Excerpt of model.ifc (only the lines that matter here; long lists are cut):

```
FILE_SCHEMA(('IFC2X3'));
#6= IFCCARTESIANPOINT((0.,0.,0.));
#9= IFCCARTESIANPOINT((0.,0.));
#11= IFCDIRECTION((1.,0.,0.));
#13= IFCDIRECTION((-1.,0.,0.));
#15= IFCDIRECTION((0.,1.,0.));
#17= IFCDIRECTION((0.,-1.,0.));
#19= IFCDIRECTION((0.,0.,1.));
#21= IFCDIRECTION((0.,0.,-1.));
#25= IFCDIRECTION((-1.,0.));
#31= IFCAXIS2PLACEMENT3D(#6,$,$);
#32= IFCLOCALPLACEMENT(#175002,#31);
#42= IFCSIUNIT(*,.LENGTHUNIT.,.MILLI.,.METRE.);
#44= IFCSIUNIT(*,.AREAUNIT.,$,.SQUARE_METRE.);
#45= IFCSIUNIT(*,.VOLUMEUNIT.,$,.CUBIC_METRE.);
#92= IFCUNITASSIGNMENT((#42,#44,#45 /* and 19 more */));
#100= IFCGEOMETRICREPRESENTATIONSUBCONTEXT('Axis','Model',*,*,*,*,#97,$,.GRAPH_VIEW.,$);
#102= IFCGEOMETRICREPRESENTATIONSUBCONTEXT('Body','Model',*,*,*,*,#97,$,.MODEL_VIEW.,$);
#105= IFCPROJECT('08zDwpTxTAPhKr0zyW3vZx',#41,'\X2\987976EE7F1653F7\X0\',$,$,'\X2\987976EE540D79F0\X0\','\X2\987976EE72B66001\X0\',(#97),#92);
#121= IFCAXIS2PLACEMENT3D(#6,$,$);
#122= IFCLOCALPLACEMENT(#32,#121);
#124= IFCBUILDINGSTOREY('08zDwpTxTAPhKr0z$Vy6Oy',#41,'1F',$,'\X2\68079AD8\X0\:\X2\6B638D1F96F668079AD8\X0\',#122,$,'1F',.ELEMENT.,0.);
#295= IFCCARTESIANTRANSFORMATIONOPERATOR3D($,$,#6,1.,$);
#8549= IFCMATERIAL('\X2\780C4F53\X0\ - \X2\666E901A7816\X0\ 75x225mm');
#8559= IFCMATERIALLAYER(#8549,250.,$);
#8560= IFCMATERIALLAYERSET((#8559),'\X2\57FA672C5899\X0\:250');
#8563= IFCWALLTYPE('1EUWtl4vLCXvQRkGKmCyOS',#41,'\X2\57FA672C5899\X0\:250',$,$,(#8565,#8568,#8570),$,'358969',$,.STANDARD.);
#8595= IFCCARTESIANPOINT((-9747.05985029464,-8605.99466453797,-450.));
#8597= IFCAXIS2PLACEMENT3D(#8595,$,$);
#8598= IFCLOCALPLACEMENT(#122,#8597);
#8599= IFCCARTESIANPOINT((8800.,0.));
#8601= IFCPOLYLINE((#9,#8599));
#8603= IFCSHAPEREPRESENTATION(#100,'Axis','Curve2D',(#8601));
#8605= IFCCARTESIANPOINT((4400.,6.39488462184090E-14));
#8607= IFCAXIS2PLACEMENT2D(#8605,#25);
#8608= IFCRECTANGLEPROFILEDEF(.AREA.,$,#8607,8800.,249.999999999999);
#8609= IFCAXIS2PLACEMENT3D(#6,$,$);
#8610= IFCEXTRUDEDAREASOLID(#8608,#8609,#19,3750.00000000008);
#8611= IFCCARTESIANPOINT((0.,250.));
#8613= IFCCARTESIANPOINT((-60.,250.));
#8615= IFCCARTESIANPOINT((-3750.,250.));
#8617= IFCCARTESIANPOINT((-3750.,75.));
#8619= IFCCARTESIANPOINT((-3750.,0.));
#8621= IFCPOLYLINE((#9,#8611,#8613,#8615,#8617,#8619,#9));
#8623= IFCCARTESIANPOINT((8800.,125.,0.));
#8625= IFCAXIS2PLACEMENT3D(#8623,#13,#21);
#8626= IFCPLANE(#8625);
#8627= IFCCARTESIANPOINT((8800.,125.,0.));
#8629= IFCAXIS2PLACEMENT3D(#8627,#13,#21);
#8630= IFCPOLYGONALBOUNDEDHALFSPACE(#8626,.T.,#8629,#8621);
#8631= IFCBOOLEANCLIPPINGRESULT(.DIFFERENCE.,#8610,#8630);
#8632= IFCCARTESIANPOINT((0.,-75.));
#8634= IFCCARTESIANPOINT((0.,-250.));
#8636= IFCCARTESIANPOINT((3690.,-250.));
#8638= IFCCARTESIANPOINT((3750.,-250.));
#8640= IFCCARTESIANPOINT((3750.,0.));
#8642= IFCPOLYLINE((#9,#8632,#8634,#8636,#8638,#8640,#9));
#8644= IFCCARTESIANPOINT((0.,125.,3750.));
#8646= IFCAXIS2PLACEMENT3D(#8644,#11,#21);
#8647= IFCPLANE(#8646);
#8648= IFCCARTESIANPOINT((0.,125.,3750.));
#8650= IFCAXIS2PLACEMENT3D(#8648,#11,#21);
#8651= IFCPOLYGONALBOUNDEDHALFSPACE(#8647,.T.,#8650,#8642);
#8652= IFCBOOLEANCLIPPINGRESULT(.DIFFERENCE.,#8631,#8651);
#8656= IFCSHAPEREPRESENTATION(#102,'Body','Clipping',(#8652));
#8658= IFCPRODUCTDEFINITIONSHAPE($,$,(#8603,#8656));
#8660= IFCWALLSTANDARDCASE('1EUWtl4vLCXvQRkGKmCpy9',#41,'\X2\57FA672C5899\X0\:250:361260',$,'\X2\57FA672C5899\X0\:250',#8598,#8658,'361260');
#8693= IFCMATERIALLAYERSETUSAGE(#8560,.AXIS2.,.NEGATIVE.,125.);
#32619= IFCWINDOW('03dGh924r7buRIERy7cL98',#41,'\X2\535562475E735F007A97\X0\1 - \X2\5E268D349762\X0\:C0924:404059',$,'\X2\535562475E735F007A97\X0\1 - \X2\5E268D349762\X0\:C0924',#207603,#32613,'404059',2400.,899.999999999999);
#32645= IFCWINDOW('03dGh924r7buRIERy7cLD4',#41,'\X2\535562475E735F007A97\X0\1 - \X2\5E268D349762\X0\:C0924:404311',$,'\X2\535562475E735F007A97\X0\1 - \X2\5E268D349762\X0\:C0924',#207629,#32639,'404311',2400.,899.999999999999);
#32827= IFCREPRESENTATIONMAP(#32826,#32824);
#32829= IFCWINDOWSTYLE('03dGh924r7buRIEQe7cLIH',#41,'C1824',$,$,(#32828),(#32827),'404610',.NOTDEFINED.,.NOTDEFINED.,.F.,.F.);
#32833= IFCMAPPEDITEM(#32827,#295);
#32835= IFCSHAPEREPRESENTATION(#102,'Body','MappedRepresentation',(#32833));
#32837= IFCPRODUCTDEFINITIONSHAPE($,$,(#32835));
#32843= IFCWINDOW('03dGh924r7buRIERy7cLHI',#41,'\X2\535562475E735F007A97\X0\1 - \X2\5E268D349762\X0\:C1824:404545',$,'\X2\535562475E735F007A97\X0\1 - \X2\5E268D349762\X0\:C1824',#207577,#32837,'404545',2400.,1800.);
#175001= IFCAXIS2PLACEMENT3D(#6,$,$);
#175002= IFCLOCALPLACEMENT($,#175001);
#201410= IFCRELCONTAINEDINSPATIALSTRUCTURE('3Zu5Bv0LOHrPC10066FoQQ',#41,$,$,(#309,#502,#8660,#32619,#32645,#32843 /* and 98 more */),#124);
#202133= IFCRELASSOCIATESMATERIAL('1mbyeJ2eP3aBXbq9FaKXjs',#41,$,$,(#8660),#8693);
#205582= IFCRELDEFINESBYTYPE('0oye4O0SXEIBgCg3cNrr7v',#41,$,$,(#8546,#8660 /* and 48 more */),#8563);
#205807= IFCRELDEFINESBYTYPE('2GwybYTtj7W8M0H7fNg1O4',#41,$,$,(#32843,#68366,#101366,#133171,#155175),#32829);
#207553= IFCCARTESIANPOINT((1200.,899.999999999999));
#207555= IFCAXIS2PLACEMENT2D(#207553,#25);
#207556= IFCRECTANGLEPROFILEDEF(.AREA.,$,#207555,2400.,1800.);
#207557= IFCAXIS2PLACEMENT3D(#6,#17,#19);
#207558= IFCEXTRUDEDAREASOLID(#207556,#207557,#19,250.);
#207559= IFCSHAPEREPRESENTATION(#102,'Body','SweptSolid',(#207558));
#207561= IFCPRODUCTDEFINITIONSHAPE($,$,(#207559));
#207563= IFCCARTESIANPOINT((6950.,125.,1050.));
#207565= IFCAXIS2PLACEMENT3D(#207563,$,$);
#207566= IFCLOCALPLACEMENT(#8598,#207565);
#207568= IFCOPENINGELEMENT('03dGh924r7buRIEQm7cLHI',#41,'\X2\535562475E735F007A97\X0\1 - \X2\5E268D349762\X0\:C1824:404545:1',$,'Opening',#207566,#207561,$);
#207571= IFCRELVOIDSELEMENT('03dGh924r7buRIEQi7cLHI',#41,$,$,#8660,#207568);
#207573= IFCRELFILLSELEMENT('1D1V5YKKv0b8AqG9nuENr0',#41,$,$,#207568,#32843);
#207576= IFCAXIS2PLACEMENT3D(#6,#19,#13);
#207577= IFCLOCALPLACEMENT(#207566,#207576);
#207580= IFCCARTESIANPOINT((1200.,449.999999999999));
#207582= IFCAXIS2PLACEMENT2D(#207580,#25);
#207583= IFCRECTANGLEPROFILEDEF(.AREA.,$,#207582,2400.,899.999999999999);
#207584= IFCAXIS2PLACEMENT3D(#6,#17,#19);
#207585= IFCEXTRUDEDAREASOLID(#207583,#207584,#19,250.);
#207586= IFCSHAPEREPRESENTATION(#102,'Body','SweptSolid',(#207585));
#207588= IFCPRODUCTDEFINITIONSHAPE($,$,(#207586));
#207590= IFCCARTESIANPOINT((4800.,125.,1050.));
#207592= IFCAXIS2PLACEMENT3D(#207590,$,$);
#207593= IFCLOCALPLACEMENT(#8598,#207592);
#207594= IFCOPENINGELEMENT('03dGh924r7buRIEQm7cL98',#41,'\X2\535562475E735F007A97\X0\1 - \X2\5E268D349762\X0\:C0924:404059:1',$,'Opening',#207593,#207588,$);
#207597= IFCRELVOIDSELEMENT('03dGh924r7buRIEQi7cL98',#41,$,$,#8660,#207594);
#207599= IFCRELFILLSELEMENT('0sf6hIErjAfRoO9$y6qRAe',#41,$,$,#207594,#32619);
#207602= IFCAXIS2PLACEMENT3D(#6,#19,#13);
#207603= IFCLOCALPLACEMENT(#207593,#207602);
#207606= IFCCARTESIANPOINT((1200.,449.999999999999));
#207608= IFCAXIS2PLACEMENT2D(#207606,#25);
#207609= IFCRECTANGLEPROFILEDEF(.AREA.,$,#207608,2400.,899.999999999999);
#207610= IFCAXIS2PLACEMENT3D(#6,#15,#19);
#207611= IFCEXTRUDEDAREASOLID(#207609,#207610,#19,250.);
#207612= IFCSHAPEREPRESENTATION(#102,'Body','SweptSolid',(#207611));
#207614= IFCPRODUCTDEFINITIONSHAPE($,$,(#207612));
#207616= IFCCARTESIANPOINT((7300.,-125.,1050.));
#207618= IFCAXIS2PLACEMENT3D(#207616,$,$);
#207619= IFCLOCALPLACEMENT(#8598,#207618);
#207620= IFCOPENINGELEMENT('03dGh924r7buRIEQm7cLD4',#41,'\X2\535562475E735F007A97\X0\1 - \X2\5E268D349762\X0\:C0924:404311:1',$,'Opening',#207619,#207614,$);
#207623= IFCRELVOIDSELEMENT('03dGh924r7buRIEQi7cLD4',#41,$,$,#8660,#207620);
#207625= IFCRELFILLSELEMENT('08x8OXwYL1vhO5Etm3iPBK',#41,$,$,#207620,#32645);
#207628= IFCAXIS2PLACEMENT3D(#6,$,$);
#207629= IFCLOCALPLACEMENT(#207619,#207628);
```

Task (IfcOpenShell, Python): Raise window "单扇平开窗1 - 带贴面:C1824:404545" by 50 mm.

```python
import numpy as np
import ifcopenshell
import ifcopenshell.api.geometry
import ifcopenshell.util.placement
import ifcopenshell.util.unit

model = ifcopenshell.open("model.ifc")
unit_scale = ifcopenshell.util.unit.calculate_unit_scale(model)

window = model.by_id(32843)
opening = window.FillsVoids[0].RelatingOpeningElement
dz = 0.05 / unit_scale

shift = np.array([0.0, 0.0, dz])
# The window is placed relative to its opening, so it follows when the opening moves.
matrix = ifcopenshell.util.placement.get_local_placement(opening.ObjectPlacement)
matrix[:3, 3] += shift
ifcopenshell.api.geometry.edit_object_placement(
    model, product=opening, matrix=matrix, is_si=False, should_transform_children=True
)

print(f"moved by {dz * unit_scale:+.3f} m")

model.write("model_updated.ifc")
```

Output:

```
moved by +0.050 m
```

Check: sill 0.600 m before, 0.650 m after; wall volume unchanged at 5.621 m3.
